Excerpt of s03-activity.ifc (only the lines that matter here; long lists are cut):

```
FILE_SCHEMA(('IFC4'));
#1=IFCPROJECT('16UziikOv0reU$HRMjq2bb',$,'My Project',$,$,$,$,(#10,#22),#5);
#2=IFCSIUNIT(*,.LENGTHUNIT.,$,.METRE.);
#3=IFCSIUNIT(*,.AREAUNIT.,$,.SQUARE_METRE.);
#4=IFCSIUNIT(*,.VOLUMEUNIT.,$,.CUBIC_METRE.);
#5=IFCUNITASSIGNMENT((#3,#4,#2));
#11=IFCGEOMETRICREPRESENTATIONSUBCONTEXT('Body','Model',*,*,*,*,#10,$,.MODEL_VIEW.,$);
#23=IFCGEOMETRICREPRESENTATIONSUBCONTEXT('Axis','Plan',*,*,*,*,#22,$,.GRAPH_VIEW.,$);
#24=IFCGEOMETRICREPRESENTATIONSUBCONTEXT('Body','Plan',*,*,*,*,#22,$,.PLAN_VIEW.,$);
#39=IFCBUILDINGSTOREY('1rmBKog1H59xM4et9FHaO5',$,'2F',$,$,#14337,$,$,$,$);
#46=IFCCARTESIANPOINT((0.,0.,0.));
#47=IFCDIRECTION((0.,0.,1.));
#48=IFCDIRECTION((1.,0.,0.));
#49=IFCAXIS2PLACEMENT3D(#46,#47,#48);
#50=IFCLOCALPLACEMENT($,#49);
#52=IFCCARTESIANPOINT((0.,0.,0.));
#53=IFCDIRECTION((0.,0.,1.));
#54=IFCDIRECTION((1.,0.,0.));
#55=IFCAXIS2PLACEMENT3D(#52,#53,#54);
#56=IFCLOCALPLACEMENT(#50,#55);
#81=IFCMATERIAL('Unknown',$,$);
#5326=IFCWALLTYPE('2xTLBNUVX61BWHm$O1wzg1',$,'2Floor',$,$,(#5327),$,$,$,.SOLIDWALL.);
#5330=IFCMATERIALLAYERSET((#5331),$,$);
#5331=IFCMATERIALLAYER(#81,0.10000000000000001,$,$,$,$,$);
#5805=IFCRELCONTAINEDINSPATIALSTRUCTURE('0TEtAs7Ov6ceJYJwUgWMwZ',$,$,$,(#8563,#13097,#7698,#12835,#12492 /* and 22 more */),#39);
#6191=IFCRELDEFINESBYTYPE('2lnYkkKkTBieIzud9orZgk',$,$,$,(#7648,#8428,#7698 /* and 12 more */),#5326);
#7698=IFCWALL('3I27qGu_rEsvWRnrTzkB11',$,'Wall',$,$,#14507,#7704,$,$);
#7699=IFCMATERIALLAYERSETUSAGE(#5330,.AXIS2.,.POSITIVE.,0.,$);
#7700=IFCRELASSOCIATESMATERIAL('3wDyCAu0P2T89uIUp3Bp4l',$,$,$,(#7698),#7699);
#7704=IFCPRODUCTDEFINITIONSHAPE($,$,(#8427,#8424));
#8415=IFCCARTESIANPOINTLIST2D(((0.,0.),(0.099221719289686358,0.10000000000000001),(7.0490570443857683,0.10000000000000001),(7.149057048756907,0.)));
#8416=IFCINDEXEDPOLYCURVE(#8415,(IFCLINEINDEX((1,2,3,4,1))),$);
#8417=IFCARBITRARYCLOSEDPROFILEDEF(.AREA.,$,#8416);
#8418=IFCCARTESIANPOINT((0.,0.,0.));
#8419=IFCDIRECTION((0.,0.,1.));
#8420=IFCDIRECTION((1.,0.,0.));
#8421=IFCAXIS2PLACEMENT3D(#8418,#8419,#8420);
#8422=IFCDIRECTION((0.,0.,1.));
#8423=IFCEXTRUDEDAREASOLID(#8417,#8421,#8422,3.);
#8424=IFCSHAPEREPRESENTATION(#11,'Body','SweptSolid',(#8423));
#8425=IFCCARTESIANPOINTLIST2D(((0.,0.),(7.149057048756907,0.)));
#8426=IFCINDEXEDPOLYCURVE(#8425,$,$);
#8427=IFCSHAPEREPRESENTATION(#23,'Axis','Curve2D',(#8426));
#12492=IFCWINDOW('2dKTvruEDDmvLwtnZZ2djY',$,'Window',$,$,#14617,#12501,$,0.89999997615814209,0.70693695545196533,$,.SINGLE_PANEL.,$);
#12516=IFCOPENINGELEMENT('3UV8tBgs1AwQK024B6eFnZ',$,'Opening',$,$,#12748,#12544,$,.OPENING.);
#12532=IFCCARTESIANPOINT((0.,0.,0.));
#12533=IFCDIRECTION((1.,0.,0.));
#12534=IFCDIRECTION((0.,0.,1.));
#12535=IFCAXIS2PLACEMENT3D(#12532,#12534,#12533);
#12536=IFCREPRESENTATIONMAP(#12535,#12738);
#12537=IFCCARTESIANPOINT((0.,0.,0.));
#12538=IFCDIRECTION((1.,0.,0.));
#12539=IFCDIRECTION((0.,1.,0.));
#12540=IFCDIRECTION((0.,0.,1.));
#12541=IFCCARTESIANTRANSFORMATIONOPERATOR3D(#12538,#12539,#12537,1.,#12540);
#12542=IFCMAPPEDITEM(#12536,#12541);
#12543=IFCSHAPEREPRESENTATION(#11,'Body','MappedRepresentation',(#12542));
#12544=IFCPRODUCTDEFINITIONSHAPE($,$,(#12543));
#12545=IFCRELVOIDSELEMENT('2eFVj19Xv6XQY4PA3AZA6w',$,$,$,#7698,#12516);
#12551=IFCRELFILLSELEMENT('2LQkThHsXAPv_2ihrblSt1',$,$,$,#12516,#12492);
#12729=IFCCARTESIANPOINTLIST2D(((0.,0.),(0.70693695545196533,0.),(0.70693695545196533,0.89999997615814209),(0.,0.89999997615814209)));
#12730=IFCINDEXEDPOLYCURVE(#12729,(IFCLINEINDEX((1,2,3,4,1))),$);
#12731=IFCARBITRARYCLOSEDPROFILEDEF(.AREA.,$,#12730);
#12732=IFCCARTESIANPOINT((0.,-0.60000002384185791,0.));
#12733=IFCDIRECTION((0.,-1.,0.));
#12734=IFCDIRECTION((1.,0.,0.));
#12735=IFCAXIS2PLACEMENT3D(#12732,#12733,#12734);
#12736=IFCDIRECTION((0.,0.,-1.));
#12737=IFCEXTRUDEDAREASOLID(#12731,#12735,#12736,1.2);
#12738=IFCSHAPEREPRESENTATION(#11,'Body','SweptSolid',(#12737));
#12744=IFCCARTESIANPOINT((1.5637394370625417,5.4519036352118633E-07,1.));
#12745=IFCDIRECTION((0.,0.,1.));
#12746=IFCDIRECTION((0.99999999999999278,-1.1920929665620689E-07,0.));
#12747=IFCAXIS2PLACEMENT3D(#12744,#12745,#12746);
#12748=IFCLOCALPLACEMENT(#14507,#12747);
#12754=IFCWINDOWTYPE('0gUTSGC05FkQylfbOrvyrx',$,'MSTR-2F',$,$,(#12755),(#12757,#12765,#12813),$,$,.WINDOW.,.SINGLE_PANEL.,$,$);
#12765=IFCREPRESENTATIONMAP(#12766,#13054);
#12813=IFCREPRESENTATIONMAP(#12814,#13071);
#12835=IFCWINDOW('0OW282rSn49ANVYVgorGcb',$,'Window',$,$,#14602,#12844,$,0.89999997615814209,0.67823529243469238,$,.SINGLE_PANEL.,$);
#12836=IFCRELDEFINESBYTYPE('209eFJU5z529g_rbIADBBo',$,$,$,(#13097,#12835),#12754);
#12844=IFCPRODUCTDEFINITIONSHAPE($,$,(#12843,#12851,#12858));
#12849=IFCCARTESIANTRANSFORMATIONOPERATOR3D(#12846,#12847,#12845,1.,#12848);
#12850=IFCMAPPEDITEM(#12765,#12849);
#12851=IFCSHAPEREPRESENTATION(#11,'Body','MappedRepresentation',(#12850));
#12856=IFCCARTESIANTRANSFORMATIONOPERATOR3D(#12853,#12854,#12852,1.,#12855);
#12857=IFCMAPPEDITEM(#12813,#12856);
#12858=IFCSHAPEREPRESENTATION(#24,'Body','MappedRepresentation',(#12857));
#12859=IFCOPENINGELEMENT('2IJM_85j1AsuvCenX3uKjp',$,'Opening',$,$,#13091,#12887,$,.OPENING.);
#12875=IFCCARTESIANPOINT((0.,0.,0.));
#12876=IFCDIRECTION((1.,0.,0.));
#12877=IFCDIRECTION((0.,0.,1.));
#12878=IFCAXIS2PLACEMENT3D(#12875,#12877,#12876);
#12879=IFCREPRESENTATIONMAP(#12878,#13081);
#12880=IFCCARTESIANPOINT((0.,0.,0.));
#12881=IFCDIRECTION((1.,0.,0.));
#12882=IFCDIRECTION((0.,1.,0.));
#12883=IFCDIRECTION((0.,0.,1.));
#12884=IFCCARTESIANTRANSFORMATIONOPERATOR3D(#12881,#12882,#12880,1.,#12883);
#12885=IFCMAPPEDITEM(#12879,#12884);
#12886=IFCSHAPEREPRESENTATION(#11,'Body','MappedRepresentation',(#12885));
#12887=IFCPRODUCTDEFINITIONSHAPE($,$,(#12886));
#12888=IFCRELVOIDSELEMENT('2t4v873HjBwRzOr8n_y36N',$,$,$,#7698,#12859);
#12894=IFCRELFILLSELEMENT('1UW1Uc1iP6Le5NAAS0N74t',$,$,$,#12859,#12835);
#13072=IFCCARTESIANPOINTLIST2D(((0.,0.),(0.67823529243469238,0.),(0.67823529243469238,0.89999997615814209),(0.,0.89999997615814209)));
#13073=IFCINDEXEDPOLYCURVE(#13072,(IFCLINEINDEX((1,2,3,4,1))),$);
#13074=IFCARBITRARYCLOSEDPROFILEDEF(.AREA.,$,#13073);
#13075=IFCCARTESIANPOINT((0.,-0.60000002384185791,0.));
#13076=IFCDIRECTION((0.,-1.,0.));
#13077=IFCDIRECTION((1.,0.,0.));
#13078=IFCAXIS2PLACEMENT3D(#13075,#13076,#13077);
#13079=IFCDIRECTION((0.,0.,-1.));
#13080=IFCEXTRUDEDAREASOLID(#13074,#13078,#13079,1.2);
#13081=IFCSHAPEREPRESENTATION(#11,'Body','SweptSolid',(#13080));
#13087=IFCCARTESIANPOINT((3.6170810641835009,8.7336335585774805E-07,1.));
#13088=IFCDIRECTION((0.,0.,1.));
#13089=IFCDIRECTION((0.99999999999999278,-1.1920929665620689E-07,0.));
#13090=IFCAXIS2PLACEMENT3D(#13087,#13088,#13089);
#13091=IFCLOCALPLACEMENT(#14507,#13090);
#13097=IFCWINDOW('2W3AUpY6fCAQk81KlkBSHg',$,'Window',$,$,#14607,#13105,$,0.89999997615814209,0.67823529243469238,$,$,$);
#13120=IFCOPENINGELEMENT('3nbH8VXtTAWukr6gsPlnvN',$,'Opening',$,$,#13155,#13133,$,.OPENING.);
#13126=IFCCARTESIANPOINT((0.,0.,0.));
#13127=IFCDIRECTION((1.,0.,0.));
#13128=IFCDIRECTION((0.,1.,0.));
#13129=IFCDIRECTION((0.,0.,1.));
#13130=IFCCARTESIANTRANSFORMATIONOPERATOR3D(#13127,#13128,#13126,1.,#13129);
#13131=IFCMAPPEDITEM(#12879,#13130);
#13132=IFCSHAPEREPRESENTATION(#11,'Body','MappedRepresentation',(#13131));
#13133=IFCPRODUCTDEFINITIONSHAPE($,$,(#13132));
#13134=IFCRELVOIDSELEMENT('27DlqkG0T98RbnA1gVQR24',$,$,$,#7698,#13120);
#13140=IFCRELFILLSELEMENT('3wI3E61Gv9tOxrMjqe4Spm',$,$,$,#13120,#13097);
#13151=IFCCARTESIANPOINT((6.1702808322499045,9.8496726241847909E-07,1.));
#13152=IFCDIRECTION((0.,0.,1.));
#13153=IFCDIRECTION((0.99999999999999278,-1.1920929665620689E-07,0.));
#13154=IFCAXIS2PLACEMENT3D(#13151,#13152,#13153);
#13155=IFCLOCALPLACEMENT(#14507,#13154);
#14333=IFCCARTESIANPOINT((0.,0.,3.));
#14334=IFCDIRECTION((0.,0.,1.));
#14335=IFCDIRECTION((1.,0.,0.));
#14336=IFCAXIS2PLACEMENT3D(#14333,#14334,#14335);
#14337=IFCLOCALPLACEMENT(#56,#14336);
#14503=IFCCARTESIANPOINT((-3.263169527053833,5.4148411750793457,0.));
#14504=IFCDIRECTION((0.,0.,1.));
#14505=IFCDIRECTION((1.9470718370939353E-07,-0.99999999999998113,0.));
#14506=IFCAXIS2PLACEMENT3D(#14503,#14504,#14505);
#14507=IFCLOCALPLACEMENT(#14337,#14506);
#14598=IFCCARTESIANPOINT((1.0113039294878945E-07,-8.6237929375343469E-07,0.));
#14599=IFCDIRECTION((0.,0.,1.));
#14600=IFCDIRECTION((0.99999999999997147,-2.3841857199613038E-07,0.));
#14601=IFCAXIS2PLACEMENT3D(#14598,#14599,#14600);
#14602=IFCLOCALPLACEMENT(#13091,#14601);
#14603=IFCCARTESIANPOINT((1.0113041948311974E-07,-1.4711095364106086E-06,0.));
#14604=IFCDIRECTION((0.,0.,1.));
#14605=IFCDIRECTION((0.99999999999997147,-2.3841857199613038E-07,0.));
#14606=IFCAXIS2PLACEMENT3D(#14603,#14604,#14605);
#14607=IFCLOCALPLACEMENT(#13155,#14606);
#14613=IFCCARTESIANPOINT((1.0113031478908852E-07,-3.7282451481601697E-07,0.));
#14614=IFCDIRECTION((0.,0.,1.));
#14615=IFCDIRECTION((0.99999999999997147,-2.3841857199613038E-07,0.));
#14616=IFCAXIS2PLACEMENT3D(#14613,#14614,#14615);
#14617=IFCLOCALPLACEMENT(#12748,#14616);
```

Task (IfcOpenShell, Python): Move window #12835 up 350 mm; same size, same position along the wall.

```python
import numpy as np
import ifcopenshell
import ifcopenshell.api.geometry
import ifcopenshell.util.placement
import ifcopenshell.util.unit

model = ifcopenshell.open("s03-activity.ifc")
unit_scale = ifcopenshell.util.unit.calculate_unit_scale(model)

window = model.by_guid("0OW282rSn49ANVYVgorGcb")
opening = window.FillsVoids[0].RelatingOpeningElement
dz = 0.35

shift = np.array([0.0, 0.0, dz])
# The window is placed relative to its opening, so it follows when the opening moves.
matrix = ifcopenshell.util.placement.get_local_placement(opening.ObjectPlacement)
matrix[:3, 3] += shift
ifcopenshell.api.geometry.edit_object_placement(
    model, product=opening, matrix=matrix, is_si=False, should_transform_children=True
)

print(f"moved by {dz * unit_scale:+.3f} m")

model.write("s03-activity_v2.ifc")
```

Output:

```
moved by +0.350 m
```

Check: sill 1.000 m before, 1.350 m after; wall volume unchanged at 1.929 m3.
